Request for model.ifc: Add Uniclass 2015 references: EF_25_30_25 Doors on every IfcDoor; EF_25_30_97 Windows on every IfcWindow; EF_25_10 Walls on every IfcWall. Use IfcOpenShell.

First a look at what the model holds.

```python
import ifcopenshell

model = ifcopenshell.open("model.ifc")
print(model.schema)
print("classifications:", [c.Name for c in model.by_type("IfcClassification")])
for ifc_class in ("IfcDoor", "IfcRoof", "IfcStair", "IfcWall", "IfcWindow"):
    print(ifc_class, len(model.by_type(ifc_class)))
```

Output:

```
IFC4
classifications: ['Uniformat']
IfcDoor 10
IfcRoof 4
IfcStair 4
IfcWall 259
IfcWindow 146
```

```python
import ifcopenshell
import ifcopenshell.api.classification

model = ifcopenshell.open("model.ifc")

system = ifcopenshell.api.classification.add_classification(model, classification="Uniclass 2015")

codes = {
    "IfcDoor": ("EF_25_30_25", "Doors"),
    "IfcWindow": ("EF_25_30_97", "Windows"),
    "IfcWall": ("EF_25_10", "Walls"),
}
for ifc_class, (code, name) in codes.items():
    products = model.by_type(ifc_class)
    ifcopenshell.api.classification.add_reference(
        model, products=products, classification=system, identification=code, name=name
    )
    print(code, len(products))

model.write("model_edited.ifc")
```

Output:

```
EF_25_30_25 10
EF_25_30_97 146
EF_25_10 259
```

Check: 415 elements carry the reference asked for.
